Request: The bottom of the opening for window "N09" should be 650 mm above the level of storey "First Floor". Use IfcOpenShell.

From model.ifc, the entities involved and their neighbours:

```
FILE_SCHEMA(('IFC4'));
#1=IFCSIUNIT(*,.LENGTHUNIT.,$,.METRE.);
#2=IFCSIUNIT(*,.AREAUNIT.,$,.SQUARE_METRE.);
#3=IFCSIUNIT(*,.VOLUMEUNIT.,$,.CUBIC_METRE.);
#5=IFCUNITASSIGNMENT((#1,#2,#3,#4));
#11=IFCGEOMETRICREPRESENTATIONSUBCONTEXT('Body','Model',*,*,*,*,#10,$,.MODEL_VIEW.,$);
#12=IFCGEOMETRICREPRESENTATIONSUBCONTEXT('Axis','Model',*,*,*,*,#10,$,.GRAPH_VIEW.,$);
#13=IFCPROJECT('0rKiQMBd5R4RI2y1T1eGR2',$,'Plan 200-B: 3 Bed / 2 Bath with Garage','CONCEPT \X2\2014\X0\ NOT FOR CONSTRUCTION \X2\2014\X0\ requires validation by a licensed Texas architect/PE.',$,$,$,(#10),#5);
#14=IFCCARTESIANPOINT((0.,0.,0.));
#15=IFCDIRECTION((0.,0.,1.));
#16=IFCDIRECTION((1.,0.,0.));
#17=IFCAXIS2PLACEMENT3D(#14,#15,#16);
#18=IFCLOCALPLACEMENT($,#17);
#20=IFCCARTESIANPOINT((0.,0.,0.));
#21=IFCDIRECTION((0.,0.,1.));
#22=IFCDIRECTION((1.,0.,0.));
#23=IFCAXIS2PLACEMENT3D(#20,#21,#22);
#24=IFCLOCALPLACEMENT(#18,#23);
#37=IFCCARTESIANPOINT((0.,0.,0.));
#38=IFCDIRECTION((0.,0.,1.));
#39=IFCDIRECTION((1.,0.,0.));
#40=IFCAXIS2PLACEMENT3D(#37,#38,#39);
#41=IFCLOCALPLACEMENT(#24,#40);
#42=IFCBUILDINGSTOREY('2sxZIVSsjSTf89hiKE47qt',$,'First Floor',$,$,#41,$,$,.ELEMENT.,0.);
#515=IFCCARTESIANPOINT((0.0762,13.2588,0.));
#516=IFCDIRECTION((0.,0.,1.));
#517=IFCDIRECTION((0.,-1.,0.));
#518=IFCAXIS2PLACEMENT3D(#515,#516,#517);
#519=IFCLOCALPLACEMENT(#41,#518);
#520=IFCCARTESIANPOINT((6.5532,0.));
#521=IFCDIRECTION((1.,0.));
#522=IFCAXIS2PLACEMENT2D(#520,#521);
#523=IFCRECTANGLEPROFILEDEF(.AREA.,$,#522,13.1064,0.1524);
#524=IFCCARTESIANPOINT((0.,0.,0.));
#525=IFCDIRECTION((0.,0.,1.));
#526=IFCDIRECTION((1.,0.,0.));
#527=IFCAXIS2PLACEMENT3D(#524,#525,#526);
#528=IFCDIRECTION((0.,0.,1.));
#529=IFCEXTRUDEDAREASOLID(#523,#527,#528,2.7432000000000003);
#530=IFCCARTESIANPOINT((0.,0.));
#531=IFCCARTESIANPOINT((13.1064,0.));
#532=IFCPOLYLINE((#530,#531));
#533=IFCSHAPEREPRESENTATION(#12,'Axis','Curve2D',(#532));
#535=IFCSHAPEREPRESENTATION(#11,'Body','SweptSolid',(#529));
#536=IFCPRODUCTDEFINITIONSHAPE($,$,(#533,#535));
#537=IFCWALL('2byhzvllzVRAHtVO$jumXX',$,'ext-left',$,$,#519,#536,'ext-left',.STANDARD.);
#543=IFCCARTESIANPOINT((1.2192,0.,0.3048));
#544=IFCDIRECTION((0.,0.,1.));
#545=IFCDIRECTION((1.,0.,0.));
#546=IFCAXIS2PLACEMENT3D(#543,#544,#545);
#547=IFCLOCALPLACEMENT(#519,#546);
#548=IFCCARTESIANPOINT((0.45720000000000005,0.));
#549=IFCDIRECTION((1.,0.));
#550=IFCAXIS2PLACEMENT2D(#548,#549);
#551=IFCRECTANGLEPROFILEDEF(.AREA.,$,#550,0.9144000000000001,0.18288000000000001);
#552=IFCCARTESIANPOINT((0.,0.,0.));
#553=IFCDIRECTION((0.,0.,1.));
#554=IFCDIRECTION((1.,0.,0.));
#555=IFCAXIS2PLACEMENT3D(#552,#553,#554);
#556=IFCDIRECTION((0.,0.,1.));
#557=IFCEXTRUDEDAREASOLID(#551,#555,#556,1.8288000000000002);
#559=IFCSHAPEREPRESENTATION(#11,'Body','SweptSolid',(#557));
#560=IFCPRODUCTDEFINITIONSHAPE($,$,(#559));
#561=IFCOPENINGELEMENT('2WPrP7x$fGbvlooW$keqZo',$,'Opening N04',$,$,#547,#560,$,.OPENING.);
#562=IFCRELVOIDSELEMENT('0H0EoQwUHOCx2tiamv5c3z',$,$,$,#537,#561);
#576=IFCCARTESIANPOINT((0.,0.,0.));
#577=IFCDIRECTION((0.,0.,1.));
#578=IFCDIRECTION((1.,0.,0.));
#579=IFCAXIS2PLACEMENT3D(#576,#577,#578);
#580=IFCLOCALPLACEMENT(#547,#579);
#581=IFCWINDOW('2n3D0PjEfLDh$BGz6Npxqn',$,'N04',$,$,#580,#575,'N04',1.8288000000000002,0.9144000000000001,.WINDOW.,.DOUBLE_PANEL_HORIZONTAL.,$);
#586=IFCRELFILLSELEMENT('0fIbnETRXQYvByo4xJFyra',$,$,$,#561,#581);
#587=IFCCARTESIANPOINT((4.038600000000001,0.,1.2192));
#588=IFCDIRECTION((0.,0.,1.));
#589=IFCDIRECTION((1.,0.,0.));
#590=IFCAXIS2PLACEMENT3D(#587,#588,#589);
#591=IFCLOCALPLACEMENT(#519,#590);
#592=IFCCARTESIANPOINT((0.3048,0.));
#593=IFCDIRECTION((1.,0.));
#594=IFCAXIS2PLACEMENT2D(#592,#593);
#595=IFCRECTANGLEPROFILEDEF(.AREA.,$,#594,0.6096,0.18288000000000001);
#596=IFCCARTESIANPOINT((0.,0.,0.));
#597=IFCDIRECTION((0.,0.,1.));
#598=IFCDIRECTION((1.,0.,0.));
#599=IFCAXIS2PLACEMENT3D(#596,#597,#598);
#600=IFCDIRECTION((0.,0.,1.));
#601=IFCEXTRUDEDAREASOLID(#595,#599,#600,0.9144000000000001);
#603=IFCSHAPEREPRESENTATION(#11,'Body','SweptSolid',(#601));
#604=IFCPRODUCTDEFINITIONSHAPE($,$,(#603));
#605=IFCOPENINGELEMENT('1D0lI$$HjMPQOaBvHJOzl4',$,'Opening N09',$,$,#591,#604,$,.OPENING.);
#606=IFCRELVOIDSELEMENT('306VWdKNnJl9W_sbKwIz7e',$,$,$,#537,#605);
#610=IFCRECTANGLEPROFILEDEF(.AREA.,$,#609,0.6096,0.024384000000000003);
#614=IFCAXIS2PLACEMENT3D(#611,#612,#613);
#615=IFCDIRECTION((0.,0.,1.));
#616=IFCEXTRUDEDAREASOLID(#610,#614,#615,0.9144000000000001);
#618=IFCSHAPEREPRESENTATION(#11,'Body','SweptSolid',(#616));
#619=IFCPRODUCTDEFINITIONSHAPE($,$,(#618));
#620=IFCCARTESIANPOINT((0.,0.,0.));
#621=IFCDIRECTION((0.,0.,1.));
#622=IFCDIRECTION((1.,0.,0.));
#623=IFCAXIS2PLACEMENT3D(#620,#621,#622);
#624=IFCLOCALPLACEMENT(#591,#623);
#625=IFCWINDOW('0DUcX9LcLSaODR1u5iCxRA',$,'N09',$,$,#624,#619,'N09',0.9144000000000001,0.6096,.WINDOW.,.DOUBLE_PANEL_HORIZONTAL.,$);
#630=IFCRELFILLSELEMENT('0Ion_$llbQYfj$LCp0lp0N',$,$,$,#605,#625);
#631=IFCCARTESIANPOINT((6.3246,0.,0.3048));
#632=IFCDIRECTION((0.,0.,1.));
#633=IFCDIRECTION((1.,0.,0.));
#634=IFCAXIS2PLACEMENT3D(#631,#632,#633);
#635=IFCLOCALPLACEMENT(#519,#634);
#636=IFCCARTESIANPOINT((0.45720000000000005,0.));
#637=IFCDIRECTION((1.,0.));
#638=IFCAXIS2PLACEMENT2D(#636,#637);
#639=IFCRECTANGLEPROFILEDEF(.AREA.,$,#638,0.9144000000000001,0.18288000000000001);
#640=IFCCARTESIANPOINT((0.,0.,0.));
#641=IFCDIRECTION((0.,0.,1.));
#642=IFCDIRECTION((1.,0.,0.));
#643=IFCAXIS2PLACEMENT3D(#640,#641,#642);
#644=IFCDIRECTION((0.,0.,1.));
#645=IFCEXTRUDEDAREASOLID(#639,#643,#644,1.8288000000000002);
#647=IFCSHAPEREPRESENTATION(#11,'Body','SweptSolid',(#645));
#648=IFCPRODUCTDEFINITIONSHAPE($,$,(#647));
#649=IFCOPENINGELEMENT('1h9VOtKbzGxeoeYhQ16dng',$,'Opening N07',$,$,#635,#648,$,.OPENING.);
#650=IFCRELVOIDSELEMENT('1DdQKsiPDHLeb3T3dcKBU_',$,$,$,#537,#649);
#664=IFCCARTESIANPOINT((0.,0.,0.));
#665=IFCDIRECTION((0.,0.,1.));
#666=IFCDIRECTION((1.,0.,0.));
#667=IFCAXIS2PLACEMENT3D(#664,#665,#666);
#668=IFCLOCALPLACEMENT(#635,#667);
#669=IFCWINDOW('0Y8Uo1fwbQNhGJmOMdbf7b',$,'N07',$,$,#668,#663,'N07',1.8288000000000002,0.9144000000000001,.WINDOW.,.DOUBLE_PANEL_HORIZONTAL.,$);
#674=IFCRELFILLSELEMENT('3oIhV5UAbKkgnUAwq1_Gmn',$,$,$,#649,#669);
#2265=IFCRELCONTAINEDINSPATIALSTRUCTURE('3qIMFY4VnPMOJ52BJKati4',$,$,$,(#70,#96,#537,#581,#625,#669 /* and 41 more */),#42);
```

```python
import numpy as np
import ifcopenshell
import ifcopenshell.api.geometry
import ifcopenshell.geom
import ifcopenshell.util.element
import ifcopenshell.util.placement
import ifcopenshell.util.shape
import ifcopenshell.util.unit

model = ifcopenshell.open("model.ifc")
unit_scale = ifcopenshell.util.unit.calculate_unit_scale(model)

window = model.by_guid("0DUcX9LcLSaODR1u5iCxRA")
opening = window.FillsVoids[0].RelatingOpeningElement
storey = ifcopenshell.util.element.get_container(window, ifc_class="IfcBuildingStorey")
level = ifcopenshell.util.placement.get_local_placement(storey.ObjectPlacement)[2, 3]

# The opening's origin need not be at the sill, so measure its lowest point.
shape = ifcopenshell.geom.create_shape(ifcopenshell.geom.settings(), opening)
bottom = ifcopenshell.util.shape.get_shape_bottom_elevation(shape, shape.geometry) / unit_scale
dz = level + 0.65 / unit_scale - bottom

shift = np.array([0.0, 0.0, dz])
# The window is placed relative to its opening, so it follows when the opening moves.
matrix = ifcopenshell.util.placement.get_local_placement(opening.ObjectPlacement)
matrix[:3, 3] += shift
ifcopenshell.api.geometry.edit_object_placement(
    model, product=opening, matrix=matrix, is_si=False, should_transform_children=True
)

print(f"moved by {dz * unit_scale:+.3f} m")

model.write("model_edited.ifc")
```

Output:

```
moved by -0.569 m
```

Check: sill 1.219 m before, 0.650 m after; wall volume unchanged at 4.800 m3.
